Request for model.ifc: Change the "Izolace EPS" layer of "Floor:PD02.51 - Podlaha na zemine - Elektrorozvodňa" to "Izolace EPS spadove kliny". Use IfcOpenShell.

First a look at what the model holds.

```python
import ifcopenshell
import ifcopenshell.util.element

model = ifcopenshell.open("model.ifc")
print(model.schema)
for layer_set in model.by_type("IfcMaterialLayerSet"):
    if layer_set.LayerSetName == "Floor:PD02.51 - Podlaha na zemine - Elektrorozvodňa":
        for layer in layer_set.MaterialLayers:
            print(layer.id(), layer.Material and layer.Material.Name, layer.LayerThickness, sep=" | ")
        print(len(ifcopenshell.util.element.get_elements_by_material(model, layer_set)), "elements and types use it")
print(sorted(m.Name for m in model.by_type("IfcMaterial") if m.Name)[:60])
```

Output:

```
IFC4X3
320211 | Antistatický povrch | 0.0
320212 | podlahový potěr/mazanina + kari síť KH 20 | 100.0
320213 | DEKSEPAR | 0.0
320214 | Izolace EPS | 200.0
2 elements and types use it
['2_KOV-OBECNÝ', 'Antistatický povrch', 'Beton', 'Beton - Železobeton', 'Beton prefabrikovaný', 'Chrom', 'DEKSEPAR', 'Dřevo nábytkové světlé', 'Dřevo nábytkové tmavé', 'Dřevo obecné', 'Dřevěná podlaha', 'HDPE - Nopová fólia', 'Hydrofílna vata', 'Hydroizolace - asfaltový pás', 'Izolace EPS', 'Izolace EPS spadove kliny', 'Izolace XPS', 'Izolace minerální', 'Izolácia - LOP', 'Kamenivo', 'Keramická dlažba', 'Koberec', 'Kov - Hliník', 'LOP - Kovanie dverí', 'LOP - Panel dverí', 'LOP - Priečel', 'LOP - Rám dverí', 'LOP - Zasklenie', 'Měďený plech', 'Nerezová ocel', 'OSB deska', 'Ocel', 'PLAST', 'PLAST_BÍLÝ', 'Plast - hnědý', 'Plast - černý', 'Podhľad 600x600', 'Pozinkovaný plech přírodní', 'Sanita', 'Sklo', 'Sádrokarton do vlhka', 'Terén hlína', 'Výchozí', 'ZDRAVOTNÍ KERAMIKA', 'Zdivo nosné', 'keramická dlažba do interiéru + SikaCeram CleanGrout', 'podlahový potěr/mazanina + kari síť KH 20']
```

```python
import ifcopenshell
import ifcopenshell.api.material

model = ifcopenshell.open("model.ifc")

layer_set = next(s for s in model.by_type("IfcMaterialLayerSet") if s.LayerSetName == "Floor:PD02.51 - Podlaha na zemine - Elektrorozvodňa")
layer = next(l for l in layer_set.MaterialLayers if l.Material and l.Material.Name == "Izolace EPS")
material = next(m for m in model.by_type("IfcMaterial") if m.Name == "Izolace EPS spadove kliny")

# Point this one layer at the other material; renaming the old one would change it everywhere.
ifcopenshell.api.material.edit_layer(model, layer=layer, attributes={"Name": material.Name}, material=material)

print([l.Material.Name if l.Material else None for l in layer_set.MaterialLayers])

model.write("model_edited.ifc")
```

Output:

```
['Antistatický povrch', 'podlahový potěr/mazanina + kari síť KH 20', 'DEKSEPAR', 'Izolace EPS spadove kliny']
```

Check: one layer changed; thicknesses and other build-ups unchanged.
